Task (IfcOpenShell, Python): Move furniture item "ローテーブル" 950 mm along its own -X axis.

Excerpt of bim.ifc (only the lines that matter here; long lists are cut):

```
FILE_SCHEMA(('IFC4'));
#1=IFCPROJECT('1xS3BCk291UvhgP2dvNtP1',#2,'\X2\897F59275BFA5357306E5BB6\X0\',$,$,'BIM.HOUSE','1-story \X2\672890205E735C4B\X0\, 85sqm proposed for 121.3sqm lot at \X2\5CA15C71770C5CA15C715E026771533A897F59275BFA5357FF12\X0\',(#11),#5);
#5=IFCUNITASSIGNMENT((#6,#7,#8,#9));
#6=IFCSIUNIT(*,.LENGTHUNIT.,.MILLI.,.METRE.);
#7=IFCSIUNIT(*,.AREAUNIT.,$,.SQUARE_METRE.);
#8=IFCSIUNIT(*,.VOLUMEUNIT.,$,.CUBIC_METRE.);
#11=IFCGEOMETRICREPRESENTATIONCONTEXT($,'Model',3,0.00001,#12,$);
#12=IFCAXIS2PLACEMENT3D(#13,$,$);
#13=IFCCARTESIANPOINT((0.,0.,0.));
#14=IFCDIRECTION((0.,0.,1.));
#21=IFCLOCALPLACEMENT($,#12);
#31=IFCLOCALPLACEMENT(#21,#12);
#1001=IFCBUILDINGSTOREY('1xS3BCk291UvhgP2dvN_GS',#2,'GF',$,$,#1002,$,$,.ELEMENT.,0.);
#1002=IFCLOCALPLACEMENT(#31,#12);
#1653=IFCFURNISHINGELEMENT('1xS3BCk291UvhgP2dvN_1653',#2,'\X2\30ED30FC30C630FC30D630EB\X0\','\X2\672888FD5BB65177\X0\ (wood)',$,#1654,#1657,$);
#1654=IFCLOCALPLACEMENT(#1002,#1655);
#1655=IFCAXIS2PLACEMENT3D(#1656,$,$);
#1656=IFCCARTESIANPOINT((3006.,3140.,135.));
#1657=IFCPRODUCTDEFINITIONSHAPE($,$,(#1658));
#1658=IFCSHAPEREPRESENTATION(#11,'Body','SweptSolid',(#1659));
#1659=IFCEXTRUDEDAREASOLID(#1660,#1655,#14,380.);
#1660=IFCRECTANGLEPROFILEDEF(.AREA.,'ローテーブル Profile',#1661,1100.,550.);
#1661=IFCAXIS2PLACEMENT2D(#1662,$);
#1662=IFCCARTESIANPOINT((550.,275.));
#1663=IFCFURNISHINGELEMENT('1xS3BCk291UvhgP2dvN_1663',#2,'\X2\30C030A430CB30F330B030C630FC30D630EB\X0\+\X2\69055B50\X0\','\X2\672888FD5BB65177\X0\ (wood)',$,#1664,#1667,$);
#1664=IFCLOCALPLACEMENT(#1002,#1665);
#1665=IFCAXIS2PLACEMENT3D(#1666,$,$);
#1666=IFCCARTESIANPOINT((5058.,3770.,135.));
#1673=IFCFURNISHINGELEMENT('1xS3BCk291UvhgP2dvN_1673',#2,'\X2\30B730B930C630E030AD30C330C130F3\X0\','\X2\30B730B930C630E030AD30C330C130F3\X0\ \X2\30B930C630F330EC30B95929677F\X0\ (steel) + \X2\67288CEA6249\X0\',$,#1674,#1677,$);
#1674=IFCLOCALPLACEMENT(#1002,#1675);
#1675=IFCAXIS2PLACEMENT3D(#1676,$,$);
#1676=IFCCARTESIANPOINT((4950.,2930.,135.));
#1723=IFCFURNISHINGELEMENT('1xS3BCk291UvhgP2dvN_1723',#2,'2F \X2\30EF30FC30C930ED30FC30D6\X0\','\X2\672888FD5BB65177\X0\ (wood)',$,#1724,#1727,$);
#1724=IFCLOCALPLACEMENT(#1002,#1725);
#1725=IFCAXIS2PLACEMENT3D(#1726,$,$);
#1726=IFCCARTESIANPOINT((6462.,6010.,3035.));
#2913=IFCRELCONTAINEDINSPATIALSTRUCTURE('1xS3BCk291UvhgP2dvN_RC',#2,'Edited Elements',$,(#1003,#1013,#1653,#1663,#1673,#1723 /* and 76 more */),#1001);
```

```python
import ifcopenshell
import ifcopenshell.api.geometry
import ifcopenshell.util.placement
import ifcopenshell.util.unit

model = ifcopenshell.open("bim.ifc")
unit_scale = ifcopenshell.util.unit.calculate_unit_scale(model)

item = model.by_guid("1xS3BCk291UvhgP2dvN_1653")
matrix = ifcopenshell.util.placement.get_local_placement(item.ObjectPlacement)
matrix[:3, 3] -= matrix[:3, 0] * 0.95 / unit_scale
ifcopenshell.api.geometry.edit_object_placement(model, product=item, matrix=matrix, is_si=False)

print(ifcopenshell.util.placement.get_local_placement(item.ObjectPlacement).round(3) + 0.0)

model.write("bim_v2.ifc")
```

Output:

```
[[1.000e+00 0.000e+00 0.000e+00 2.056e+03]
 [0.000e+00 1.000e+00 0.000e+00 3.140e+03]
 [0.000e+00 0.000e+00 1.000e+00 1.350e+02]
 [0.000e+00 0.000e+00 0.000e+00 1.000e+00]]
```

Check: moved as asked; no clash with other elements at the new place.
